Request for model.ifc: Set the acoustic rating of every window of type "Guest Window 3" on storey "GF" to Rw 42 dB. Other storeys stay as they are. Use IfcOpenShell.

First a look at what the model holds.

```python
import ifcopenshell
import ifcopenshell.util.element

model = ifcopenshell.open("model.ifc")
print(model.schema)
storey = next(s for s in model.by_type("IfcBuildingStorey") if s.Name == "GF")
windows = [e for e in ifcopenshell.util.element.get_decomposition(storey) if e.is_a("IfcWindow")]
seen = {}
for e in windows:
    element_type = ifcopenshell.util.element.get_type(e)
    key = (element_type.Name if element_type != e and element_type else None, ifcopenshell.util.element.get_pset(e, "Pset_WindowCommon", "AcousticRating"))
    seen[key] = seen.get(key, 0) + 1
for (name, value), count in sorted(seen.items(), key=str):
    print(count, "x", name, "|", value)
```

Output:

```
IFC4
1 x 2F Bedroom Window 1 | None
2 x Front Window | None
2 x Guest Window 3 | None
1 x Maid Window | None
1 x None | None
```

```python
import ifcopenshell
import ifcopenshell.api.pset
import ifcopenshell.util.element

model = ifcopenshell.open("model.ifc")

storey = next(s for s in model.by_type("IfcBuildingStorey") if s.Name == "GF")
windows = [e for e in ifcopenshell.util.element.get_decomposition(storey) if e.is_a("IfcWindow")]

count = 0
for e in windows:
    element_type = ifcopenshell.util.element.get_type(e)
    if element_type in (None, e) or element_type.Name != "Guest Window 3":
        continue
    # add_pset returns the element's existing set when there is one.
    pset = ifcopenshell.api.pset.add_pset(model, product=e, name="Pset_WindowCommon")
    ifcopenshell.api.pset.edit_pset(model, pset=pset, properties={"AcousticRating": "Rw 42 dB"})
    count += 1

print(count, "windows updated")

model.write("model_v2.ifc")
```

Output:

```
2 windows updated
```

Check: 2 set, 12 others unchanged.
